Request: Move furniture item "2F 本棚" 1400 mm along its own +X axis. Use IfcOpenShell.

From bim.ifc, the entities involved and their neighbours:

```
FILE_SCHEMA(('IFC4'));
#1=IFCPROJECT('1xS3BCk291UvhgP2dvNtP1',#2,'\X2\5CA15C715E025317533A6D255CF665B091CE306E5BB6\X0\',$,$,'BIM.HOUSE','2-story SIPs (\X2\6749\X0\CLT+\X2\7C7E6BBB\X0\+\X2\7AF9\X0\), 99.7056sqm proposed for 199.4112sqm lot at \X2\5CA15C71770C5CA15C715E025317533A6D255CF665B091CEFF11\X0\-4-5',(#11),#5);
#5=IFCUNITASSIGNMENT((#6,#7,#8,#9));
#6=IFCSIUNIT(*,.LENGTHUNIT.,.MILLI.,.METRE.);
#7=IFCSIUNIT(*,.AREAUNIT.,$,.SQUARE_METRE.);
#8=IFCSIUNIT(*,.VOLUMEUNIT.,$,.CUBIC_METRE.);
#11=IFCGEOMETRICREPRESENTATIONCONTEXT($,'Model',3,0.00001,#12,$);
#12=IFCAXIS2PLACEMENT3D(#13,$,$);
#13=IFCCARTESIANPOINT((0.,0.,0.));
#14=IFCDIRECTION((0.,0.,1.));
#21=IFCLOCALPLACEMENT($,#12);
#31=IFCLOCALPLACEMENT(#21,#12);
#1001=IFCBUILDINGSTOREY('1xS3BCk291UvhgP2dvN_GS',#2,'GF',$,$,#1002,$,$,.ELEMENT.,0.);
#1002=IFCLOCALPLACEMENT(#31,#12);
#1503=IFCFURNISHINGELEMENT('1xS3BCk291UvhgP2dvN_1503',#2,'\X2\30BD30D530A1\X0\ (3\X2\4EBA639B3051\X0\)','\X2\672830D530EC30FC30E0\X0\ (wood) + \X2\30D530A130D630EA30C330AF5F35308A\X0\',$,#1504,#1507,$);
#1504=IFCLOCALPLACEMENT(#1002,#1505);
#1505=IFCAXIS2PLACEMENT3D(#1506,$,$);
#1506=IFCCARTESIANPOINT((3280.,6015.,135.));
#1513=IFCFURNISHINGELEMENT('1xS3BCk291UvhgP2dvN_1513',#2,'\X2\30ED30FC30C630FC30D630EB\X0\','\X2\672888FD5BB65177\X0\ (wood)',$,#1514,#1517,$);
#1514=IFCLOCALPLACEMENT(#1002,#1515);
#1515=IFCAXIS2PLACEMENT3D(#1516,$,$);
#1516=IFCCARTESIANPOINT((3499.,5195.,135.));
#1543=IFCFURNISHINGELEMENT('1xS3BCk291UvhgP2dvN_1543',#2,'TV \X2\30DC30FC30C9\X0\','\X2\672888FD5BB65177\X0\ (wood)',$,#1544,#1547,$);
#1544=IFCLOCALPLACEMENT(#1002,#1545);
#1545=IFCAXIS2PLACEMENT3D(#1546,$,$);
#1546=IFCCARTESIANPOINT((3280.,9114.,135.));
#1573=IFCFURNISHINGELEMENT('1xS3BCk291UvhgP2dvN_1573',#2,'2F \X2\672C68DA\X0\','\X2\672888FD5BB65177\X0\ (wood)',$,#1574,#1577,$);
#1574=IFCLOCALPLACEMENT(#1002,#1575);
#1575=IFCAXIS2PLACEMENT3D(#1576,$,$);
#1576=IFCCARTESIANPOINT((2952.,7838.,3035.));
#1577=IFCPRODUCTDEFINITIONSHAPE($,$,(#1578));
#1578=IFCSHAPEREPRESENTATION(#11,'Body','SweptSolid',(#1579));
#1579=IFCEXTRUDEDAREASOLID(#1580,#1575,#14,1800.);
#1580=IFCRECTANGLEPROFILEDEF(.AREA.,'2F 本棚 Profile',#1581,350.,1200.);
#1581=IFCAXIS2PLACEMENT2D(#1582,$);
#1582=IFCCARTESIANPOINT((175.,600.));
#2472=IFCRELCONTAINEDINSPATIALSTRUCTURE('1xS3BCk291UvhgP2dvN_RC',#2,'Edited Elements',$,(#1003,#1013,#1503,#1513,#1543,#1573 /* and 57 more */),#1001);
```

```python
import ifcopenshell
import ifcopenshell.api.geometry
import ifcopenshell.util.placement

model = ifcopenshell.open("bim.ifc")

item = model.by_id(1573)
matrix = ifcopenshell.util.placement.get_local_placement(item.ObjectPlacement)
matrix[:3, 3] += matrix[:3, 0] * 1400.0
ifcopenshell.api.geometry.edit_object_placement(model, product=item, matrix=matrix, is_si=False)

print(ifcopenshell.util.placement.get_local_placement(item.ObjectPlacement).round(3) + 0.0)

model.write("bim_v2.ifc")
```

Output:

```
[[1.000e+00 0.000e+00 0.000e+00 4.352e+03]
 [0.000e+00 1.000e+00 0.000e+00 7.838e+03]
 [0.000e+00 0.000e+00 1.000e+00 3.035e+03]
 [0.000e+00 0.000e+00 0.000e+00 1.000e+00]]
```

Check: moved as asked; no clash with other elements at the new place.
